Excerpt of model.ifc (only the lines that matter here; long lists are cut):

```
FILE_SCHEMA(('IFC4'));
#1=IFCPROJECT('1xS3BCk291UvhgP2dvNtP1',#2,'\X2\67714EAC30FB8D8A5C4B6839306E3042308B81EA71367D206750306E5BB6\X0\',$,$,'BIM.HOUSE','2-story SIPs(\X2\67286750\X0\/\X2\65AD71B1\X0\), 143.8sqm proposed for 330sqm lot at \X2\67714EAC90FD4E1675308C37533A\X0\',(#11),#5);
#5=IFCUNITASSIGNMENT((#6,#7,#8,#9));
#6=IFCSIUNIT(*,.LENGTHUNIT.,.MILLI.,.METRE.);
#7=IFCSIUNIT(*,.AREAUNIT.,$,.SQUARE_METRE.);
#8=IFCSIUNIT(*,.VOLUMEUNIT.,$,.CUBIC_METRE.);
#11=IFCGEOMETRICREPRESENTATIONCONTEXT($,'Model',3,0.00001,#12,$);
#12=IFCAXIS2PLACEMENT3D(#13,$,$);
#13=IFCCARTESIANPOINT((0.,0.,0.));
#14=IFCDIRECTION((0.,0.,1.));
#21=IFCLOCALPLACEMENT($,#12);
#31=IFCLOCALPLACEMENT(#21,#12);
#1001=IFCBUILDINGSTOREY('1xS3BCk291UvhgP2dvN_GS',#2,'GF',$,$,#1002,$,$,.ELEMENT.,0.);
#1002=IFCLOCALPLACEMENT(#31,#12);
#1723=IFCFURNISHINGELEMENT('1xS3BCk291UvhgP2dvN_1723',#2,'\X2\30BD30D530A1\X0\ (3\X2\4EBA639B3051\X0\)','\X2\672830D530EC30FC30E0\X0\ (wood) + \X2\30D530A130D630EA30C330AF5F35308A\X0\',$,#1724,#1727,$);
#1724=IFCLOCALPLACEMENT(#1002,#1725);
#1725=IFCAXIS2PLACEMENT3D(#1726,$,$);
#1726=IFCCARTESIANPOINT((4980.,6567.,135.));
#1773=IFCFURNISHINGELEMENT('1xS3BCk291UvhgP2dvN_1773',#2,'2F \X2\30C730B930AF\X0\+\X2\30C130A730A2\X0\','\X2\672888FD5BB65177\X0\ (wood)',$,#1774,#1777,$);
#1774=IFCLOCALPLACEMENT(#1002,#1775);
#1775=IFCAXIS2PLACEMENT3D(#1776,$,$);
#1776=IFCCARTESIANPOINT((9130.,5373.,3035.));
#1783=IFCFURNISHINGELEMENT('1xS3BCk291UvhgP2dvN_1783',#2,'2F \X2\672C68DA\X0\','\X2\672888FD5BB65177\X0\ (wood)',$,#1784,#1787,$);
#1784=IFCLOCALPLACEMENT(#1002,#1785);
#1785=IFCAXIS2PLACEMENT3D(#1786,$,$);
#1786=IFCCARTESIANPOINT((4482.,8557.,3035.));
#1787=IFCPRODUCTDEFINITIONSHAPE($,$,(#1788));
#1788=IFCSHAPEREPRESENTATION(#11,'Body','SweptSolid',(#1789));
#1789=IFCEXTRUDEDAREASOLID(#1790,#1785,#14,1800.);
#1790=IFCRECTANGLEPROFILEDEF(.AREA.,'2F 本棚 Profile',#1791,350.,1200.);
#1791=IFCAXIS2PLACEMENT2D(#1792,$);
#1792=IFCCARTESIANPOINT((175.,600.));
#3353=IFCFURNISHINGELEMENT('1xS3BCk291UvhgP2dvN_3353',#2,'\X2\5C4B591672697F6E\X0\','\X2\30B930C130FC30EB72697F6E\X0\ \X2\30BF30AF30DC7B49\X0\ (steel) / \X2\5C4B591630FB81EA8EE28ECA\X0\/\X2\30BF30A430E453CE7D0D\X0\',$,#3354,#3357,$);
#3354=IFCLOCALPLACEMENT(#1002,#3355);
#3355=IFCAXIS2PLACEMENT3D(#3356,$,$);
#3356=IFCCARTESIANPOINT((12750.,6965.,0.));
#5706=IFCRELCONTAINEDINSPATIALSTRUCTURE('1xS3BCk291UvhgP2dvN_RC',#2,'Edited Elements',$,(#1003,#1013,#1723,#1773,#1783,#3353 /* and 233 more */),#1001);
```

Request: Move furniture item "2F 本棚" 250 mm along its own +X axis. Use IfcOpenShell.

```python
import ifcopenshell
import ifcopenshell.api.geometry
import ifcopenshell.util.placement

model = ifcopenshell.open("model.ifc")

item = model.by_id(1783)
matrix = ifcopenshell.util.placement.get_local_placement(item.ObjectPlacement)
matrix[:3, 3] += matrix[:3, 0] * 250.0
ifcopenshell.api.geometry.edit_object_placement(model, product=item, matrix=matrix, is_si=False)

print(ifcopenshell.util.placement.get_local_placement(item.ObjectPlacement).round(3) + 0.0)

model.write("model-out.ifc")
```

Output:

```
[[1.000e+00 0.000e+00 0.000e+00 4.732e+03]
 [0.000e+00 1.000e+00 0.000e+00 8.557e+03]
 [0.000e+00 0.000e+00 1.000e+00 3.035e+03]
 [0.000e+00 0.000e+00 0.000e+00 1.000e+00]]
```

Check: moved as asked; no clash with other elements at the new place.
